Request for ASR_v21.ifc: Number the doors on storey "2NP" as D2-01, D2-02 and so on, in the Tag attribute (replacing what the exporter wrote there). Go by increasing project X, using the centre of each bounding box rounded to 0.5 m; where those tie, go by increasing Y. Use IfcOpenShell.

First a look at what the model holds.

```python
import ifcopenshell
import ifcopenshell.util.element
import ifcopenshell.util.placement

model = ifcopenshell.open("ASR_v21.ifc")
print(model.schema)
storey = next(s for s in model.by_type("IfcBuildingStorey") if s.Name == "2NP")
doors = [e for e in ifcopenshell.util.element.get_decomposition(storey) if e.is_a("IfcDoor")]
for e in sorted(doors, key=lambda e: e.id()):
    origin = ifcopenshell.util.placement.get_local_placement(e.ObjectPlacement)[:3, 3]
    print(e.id(), e.Tag, e.Name, origin.round(2) + 0.0, sep=" | ")
```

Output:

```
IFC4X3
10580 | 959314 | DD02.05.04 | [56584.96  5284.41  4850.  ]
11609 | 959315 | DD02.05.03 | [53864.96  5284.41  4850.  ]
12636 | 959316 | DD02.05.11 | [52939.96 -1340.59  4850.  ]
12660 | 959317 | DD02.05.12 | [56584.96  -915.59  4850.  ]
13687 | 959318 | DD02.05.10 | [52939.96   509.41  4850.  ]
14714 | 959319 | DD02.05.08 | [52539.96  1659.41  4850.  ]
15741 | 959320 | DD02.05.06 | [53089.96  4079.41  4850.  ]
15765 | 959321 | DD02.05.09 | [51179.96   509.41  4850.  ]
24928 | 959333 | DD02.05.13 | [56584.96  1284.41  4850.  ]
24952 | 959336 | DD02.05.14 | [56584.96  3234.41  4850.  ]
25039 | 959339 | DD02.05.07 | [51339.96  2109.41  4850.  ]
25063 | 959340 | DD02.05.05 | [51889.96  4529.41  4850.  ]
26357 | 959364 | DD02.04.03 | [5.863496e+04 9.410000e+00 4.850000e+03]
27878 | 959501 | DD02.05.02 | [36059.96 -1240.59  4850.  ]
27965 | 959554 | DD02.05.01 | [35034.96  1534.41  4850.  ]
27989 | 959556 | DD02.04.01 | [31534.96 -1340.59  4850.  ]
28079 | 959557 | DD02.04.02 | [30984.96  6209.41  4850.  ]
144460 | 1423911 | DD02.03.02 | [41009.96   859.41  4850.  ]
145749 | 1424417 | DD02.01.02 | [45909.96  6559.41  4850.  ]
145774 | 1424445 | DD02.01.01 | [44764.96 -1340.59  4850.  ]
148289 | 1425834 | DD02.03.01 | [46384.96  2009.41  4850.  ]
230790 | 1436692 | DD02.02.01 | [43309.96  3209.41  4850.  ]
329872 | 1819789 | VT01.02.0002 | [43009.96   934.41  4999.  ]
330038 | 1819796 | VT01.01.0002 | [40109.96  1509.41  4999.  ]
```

```python
import ifcopenshell
import ifcopenshell.geom
import ifcopenshell.util.element
import ifcopenshell.util.shape

model = ifcopenshell.open("ASR_v21.ifc")
settings = ifcopenshell.geom.settings()
settings.set("use-world-coords", True)


def centre(element):
    shape = ifcopenshell.geom.create_shape(settings, element)
    return ifcopenshell.util.shape.get_bbox_centroid(shape.geometry)


storey = next(s for s in model.by_type("IfcBuildingStorey") if s.Name == "2NP")
doors = [e for e in ifcopenshell.util.element.get_decomposition(storey) if e.is_a("IfcDoor")]

# Insertion points can sit at a corner or the storey origin, so sort by the geometry (in metres).
centres = {e: centre(e) for e in doors}
doors.sort(key=lambda e: (round(centres[e][0] / 0.5), centres[e][1]))

for i, e in enumerate(doors, start=1):
    number = f"D2-{i:02d}"
    e.Tag = number
    print(e.id(), number)

model.write("ASR_v21-out.ifc")
```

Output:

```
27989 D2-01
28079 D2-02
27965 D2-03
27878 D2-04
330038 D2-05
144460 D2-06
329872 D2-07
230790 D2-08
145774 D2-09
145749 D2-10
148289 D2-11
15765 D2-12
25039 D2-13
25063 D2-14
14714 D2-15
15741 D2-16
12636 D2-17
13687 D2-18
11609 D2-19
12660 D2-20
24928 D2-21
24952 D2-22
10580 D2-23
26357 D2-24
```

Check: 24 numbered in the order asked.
